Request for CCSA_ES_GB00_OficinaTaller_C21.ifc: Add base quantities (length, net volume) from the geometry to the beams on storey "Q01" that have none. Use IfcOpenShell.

First a look at what the model holds.

```python
import ifcopenshell
import ifcopenshell.util.element
import ifcopenshell.util.unit

model = ifcopenshell.open("CCSA_ES_GB00_OficinaTaller_C21.ifc")
print(model.schema)
for unit_type in ("LENGTHUNIT", "AREAUNIT", "VOLUMEUNIT"):
    print(unit_type, ifcopenshell.util.unit.calculate_unit_scale(model, unit_type))
storey = next(s for s in model.by_type("IfcBuildingStorey") if s.Name == "Q01")
beams = [e for e in ifcopenshell.util.element.get_decomposition(storey) if e.is_a("IfcBeam")]
for e in sorted(beams, key=lambda e: e.id()):
    print(e.id(), e.is_a(), e.Name, list(ifcopenshell.util.element.get_psets(e, qtos_only=True)), sep=" | ")
```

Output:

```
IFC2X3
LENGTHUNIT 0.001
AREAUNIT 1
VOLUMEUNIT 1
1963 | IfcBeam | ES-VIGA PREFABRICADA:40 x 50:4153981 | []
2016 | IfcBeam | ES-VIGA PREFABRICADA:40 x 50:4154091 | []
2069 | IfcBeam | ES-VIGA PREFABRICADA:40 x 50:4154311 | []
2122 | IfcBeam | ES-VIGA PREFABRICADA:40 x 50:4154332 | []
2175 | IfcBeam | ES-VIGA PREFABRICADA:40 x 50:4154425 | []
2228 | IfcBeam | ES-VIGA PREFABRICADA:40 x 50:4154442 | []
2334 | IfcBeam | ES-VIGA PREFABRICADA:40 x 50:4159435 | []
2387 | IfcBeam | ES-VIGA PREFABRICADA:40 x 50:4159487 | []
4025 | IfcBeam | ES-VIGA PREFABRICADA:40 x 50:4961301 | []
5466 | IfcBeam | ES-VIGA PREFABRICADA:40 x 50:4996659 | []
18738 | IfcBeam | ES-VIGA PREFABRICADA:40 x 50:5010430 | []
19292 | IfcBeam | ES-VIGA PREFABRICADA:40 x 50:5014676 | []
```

```python
import ifcopenshell
import ifcopenshell.api.pset
import ifcopenshell.geom
import ifcopenshell.util.element
import ifcopenshell.util.shape
import ifcopenshell.util.unit

model = ifcopenshell.open("CCSA_ES_GB00_OficinaTaller_C21.ifc")
unit_scale = ifcopenshell.util.unit.calculate_unit_scale(model)
volume_scale = ifcopenshell.util.unit.calculate_unit_scale(model, "VOLUMEUNIT")
settings = ifcopenshell.geom.settings()

storey = next(s for s in model.by_type("IfcBuildingStorey") if s.Name == "Q01")
beams = [e for e in ifcopenshell.util.element.get_decomposition(storey) if e.is_a("IfcBeam")]

for e in sorted(beams, key=lambda e: e.id()):
    if ifcopenshell.util.element.get_psets(e, qtos_only=True, should_inherit=False):
        continue
    # Geometry comes back in metres, in the element's own axes.
    shape = ifcopenshell.geom.create_shape(settings, e)
    values = {
        "Length": ifcopenshell.util.shape.get_max_xyz(shape.geometry) / unit_scale,
        "NetVolume": ifcopenshell.util.shape.get_volume(shape.geometry) / volume_scale,
    }
    qto = ifcopenshell.api.pset.add_qto(model, product=e, name="BaseQuantities")
    ifcopenshell.api.pset.edit_qto(model, qto=qto, properties=values)
    print(e.id(), {k: round(v, 3) for k, v in values.items()})

model.write("CCSA_ES_GB00_OficinaTaller_C21_updated.ifc")
```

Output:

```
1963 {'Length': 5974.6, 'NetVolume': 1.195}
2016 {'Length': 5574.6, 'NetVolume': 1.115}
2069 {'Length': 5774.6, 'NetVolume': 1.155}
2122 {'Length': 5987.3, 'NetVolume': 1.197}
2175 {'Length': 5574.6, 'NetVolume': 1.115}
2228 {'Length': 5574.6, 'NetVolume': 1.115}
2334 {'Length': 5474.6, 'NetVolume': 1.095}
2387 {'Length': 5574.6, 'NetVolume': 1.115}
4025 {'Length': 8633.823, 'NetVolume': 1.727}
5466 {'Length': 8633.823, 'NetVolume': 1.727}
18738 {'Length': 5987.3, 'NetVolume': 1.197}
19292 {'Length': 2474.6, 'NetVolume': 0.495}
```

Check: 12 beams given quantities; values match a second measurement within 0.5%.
